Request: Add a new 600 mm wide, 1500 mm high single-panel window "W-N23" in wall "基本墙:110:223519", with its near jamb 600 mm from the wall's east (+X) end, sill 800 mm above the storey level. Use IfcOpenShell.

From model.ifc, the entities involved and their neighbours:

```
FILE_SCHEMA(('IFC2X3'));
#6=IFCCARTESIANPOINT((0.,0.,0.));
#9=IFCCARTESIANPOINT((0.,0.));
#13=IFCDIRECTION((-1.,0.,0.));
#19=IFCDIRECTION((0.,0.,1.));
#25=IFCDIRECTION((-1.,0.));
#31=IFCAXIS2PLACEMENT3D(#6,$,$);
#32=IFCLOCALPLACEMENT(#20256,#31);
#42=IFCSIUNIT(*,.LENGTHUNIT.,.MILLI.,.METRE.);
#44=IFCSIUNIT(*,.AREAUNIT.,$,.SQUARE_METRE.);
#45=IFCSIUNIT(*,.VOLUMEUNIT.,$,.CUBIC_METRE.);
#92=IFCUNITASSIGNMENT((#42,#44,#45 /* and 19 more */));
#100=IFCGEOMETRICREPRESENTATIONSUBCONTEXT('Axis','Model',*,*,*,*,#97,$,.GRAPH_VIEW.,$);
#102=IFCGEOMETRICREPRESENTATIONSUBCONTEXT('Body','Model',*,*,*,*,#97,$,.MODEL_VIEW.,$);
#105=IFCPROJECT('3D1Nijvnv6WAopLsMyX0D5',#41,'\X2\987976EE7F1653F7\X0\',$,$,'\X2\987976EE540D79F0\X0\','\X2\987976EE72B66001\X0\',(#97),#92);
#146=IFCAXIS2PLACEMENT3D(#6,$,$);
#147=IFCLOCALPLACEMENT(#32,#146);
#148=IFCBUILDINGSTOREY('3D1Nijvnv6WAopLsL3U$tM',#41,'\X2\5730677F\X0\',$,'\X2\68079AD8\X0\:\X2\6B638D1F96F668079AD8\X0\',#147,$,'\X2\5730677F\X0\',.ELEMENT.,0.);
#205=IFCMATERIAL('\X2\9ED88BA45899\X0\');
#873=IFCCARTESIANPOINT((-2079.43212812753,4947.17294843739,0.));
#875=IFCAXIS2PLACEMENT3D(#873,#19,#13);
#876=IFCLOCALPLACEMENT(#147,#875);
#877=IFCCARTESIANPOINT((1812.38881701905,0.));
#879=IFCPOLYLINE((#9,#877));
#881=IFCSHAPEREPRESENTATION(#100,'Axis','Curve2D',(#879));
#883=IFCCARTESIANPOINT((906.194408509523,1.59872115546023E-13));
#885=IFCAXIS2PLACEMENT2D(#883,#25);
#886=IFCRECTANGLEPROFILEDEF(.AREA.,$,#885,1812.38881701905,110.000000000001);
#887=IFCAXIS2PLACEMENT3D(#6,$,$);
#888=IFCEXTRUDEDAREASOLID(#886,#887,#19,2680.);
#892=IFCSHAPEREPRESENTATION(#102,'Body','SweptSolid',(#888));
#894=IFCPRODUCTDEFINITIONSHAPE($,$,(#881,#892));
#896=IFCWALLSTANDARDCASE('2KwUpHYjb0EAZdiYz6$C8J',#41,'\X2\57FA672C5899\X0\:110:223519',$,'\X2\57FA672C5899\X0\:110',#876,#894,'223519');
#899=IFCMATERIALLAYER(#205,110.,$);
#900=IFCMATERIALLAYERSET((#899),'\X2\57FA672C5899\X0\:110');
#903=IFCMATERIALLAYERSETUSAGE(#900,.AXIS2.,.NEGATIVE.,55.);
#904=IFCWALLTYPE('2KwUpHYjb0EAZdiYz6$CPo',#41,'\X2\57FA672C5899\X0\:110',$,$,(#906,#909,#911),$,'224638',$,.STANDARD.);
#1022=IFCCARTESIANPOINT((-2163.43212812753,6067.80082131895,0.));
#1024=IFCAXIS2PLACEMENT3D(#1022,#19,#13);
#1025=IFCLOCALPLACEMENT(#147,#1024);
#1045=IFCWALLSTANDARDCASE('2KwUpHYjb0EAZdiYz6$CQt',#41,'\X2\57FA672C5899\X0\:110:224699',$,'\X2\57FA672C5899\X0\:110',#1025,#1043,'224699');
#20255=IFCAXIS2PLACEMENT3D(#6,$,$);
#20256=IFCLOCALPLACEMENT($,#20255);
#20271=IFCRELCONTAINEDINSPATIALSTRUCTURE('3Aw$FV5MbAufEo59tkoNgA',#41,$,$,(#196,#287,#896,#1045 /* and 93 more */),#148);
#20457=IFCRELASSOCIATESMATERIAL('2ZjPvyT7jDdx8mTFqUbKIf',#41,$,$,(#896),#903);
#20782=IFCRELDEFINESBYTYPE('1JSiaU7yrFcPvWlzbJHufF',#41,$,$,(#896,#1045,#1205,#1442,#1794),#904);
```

```python
import numpy as np
import ifcopenshell
import ifcopenshell.api.feature
import ifcopenshell.api.geometry
import ifcopenshell.api.root
import ifcopenshell.api.spatial
import ifcopenshell.api.type
import ifcopenshell.geom
import ifcopenshell.util.element
import ifcopenshell.util.placement
import ifcopenshell.util.representation
import ifcopenshell.util.shape
import ifcopenshell.util.unit

model = ifcopenshell.open("model.ifc")
unit_scale = ifcopenshell.util.unit.calculate_unit_scale(model)
settings = ifcopenshell.geom.settings()


def volume(element):
    """Net volume in cubic metres, openings subtracted."""
    shape = ifcopenshell.geom.create_shape(settings, element)
    return ifcopenshell.util.shape.get_volume(shape.geometry)


wall = model.by_id(896)
storey = ifcopenshell.util.element.get_container(wall, ifc_class="IfcBuildingStorey")
context = ifcopenshell.util.representation.get_context(model, "Model", "Body", "MODEL_VIEW")
before = volume(wall)

width, height, from_end, sill = 0.6, 1.5, 0.6, 0.8  # metres

# The wall runs along its own X axis, and the end named is its -X end.
wall_shape = ifcopenshell.geom.create_shape(settings, wall)
x, y, z = ifcopenshell.util.shape.get_vertices(wall_shape.geometry).T
start = x.min() + from_end
face, thickness = float(y.min()), float(y.max() - y.min())
wall_matrix = ifcopenshell.util.placement.get_local_placement(wall.ObjectPlacement)
level = ifcopenshell.util.placement.get_local_placement(storey.ObjectPlacement)[2, 3]


def in_wall(x, y):
    """Placement at x, y metres in the wall's axes, at sill height."""
    matrix = wall_matrix.copy()
    matrix[:, 3] = wall_matrix @ np.array([x / unit_scale, y / unit_scale, 0.0, 1.0])
    matrix[2, 3] = level + sill / unit_scale
    return matrix


# Opening: a box that overshoots both wall faces by 50 mm.
opening = ifcopenshell.api.root.create_entity(model, ifc_class="IfcOpeningElement")
box = ifcopenshell.api.geometry.add_wall_representation(
    model, context=context, length=width, height=height, thickness=thickness + 0.1
)
ifcopenshell.api.geometry.assign_representation(model, product=opening, representation=box)
ifcopenshell.api.geometry.edit_object_placement(model, product=opening, matrix=in_wall(start, face - 0.05), is_si=False)
ifcopenshell.api.feature.add_feature(model, feature=opening, element=wall)

window = ifcopenshell.api.root.create_entity(model, ifc_class="IfcWindow", name="W-N23")
window.OverallWidth, window.OverallHeight = width / unit_scale, height / unit_scale
body = ifcopenshell.api.geometry.add_window_representation(
    model,
    context=context,
    overall_width=window.OverallWidth,
    overall_height=window.OverallHeight,
    partition_type="SINGLE_PANEL",
)
ifcopenshell.api.geometry.assign_representation(model, product=window, representation=body)
ifcopenshell.api.spatial.assign_container(model, products=[window], relating_structure=storey)
fills = ifcopenshell.api.feature.add_filling(model, opening=opening, element=window)
fills.OwnerHistory = window.OwnerHistory  # required in IFC2X3

# IFC2X3 keeps the operation on the window style.
style = ifcopenshell.api.root.create_entity(model, ifc_class="IfcWindowStyle", name="W-N23")
style.OperationType, style.ConstructionType = "SINGLE_PANEL", "NOTDEFINED"
style.ParameterTakesPrecedence = style.Sizeable = False
ifcopenshell.api.type.assign_type(model, related_objects=[window], relating_type=style)

# Centre the window in the wall's thickness.
ifcopenshell.api.geometry.edit_object_placement(model, product=window, matrix=in_wall(start, face), is_si=False)
window_shape = ifcopenshell.geom.create_shape(settings, window)
depth = ifcopenshell.util.shape.get_vertices(window_shape.geometry)[:, 1]
offset = face + thickness / 2 - (depth.min() + depth.max()) / 2
ifcopenshell.api.geometry.edit_object_placement(model, product=window, matrix=in_wall(start, offset), is_si=False)

after = volume(wall)

print(f"wall volume {before:.3f} -> {after:.3f} m3")

model.write("model_edited.ifc")
```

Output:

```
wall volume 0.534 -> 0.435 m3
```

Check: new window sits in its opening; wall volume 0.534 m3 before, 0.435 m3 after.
